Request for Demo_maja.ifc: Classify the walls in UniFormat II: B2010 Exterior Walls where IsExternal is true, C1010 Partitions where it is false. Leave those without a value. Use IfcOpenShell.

First a look at what the model holds.

```python
import ifcopenshell
import ifcopenshell.util.element

model = ifcopenshell.open("Demo_maja.ifc")
print(model.schema)
print("classifications:", [c.Name for c in model.by_type("IfcClassification")])
values = [ifcopenshell.util.element.get_pset(e, "Pset_WallCommon", "IsExternal") for e in model.by_type("IfcWall")]
for value in (True, False, None):
    print("IsExternal", value, values.count(value))
```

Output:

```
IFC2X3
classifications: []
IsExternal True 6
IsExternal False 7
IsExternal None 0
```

```python
import ifcopenshell
import ifcopenshell.api.classification
import ifcopenshell.util.element

model = ifcopenshell.open("Demo_maja.ifc")

# IFC2X3 requires Source and Edition and has no link from the project to the system.
system = model.create_entity("IfcClassification", Source="ASTM", Edition="E1557", Name="UniFormat II")

walls = model.by_type("IfcWall")
external = {e: ifcopenshell.util.element.get_pset(e, "Pset_WallCommon", "IsExternal") for e in walls}
for flag, code, name in ((True, "B2010", "Exterior Walls"), (False, "C1010", "Partitions")):
    products = [e for e in walls if external[e] is flag]
    ifcopenshell.api.classification.add_reference(
        model, products=products, classification=system, identification=code, name=name
    )
    print(code, len(products))

model.write("Demo_maja_updated.ifc")
```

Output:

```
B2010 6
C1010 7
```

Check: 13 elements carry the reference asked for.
